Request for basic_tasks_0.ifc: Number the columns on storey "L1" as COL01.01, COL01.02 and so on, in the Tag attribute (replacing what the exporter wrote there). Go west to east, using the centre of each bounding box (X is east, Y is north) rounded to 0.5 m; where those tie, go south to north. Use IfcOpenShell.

First a look at what the model holds.

```python
import ifcopenshell
import ifcopenshell.util.element
import ifcopenshell.util.placement

model = ifcopenshell.open("basic_tasks_0.ifc")
print(model.schema)
storey = next(s for s in model.by_type("IfcBuildingStorey") if s.Name == "L1")
columns = [e for e in ifcopenshell.util.element.get_decomposition(storey) if e.is_a("IfcColumn")]
for e in sorted(columns, key=lambda e: e.id()):
    origin = ifcopenshell.util.placement.get_local_placement(e.ObjectPlacement)[:3, 3]
    print(e.id(), e.Tag, e.Name, origin.round(2) + 0.0, sep=" | ")
```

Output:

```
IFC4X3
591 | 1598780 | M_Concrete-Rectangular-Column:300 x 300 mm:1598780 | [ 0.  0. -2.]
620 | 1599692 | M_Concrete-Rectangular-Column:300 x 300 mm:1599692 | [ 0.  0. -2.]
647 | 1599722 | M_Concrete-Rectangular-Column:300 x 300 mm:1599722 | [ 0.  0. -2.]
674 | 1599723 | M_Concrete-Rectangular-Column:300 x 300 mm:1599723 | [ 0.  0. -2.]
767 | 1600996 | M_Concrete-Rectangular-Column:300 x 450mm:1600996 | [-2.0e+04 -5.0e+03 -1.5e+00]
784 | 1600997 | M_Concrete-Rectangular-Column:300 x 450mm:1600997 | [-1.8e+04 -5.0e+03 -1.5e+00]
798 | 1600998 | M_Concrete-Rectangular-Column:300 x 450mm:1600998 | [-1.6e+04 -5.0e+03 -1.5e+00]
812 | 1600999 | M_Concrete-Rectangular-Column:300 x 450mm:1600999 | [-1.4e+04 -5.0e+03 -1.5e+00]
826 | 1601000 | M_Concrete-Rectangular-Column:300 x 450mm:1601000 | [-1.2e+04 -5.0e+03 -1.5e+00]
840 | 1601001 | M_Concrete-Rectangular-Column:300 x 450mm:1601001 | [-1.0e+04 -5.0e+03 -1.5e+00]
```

```python
import ifcopenshell
import ifcopenshell.geom
import ifcopenshell.util.element
import ifcopenshell.util.shape

model = ifcopenshell.open("basic_tasks_0.ifc")
settings = ifcopenshell.geom.settings()
settings.set("use-world-coords", True)


def centre(element):
    shape = ifcopenshell.geom.create_shape(settings, element)
    return ifcopenshell.util.shape.get_bbox_centroid(shape.geometry)


storey = next(s for s in model.by_type("IfcBuildingStorey") if s.Name == "L1")
columns = [e for e in ifcopenshell.util.element.get_decomposition(storey) if e.is_a("IfcColumn")]

# Insertion points can sit at a corner or the storey origin, so sort by the geometry (in metres).
centres = {e: centre(e) for e in columns}
columns.sort(key=lambda e: (round(centres[e][0] / 0.5), centres[e][1]))

for i, e in enumerate(columns, start=1):
    number = f"COL01.{i:02d}"
    e.Tag = number
    print(e.id(), number)

model.write("basic_tasks_0_edited.ifc")
```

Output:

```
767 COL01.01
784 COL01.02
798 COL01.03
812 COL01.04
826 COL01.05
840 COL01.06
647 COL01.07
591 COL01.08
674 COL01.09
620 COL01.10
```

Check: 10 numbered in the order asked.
